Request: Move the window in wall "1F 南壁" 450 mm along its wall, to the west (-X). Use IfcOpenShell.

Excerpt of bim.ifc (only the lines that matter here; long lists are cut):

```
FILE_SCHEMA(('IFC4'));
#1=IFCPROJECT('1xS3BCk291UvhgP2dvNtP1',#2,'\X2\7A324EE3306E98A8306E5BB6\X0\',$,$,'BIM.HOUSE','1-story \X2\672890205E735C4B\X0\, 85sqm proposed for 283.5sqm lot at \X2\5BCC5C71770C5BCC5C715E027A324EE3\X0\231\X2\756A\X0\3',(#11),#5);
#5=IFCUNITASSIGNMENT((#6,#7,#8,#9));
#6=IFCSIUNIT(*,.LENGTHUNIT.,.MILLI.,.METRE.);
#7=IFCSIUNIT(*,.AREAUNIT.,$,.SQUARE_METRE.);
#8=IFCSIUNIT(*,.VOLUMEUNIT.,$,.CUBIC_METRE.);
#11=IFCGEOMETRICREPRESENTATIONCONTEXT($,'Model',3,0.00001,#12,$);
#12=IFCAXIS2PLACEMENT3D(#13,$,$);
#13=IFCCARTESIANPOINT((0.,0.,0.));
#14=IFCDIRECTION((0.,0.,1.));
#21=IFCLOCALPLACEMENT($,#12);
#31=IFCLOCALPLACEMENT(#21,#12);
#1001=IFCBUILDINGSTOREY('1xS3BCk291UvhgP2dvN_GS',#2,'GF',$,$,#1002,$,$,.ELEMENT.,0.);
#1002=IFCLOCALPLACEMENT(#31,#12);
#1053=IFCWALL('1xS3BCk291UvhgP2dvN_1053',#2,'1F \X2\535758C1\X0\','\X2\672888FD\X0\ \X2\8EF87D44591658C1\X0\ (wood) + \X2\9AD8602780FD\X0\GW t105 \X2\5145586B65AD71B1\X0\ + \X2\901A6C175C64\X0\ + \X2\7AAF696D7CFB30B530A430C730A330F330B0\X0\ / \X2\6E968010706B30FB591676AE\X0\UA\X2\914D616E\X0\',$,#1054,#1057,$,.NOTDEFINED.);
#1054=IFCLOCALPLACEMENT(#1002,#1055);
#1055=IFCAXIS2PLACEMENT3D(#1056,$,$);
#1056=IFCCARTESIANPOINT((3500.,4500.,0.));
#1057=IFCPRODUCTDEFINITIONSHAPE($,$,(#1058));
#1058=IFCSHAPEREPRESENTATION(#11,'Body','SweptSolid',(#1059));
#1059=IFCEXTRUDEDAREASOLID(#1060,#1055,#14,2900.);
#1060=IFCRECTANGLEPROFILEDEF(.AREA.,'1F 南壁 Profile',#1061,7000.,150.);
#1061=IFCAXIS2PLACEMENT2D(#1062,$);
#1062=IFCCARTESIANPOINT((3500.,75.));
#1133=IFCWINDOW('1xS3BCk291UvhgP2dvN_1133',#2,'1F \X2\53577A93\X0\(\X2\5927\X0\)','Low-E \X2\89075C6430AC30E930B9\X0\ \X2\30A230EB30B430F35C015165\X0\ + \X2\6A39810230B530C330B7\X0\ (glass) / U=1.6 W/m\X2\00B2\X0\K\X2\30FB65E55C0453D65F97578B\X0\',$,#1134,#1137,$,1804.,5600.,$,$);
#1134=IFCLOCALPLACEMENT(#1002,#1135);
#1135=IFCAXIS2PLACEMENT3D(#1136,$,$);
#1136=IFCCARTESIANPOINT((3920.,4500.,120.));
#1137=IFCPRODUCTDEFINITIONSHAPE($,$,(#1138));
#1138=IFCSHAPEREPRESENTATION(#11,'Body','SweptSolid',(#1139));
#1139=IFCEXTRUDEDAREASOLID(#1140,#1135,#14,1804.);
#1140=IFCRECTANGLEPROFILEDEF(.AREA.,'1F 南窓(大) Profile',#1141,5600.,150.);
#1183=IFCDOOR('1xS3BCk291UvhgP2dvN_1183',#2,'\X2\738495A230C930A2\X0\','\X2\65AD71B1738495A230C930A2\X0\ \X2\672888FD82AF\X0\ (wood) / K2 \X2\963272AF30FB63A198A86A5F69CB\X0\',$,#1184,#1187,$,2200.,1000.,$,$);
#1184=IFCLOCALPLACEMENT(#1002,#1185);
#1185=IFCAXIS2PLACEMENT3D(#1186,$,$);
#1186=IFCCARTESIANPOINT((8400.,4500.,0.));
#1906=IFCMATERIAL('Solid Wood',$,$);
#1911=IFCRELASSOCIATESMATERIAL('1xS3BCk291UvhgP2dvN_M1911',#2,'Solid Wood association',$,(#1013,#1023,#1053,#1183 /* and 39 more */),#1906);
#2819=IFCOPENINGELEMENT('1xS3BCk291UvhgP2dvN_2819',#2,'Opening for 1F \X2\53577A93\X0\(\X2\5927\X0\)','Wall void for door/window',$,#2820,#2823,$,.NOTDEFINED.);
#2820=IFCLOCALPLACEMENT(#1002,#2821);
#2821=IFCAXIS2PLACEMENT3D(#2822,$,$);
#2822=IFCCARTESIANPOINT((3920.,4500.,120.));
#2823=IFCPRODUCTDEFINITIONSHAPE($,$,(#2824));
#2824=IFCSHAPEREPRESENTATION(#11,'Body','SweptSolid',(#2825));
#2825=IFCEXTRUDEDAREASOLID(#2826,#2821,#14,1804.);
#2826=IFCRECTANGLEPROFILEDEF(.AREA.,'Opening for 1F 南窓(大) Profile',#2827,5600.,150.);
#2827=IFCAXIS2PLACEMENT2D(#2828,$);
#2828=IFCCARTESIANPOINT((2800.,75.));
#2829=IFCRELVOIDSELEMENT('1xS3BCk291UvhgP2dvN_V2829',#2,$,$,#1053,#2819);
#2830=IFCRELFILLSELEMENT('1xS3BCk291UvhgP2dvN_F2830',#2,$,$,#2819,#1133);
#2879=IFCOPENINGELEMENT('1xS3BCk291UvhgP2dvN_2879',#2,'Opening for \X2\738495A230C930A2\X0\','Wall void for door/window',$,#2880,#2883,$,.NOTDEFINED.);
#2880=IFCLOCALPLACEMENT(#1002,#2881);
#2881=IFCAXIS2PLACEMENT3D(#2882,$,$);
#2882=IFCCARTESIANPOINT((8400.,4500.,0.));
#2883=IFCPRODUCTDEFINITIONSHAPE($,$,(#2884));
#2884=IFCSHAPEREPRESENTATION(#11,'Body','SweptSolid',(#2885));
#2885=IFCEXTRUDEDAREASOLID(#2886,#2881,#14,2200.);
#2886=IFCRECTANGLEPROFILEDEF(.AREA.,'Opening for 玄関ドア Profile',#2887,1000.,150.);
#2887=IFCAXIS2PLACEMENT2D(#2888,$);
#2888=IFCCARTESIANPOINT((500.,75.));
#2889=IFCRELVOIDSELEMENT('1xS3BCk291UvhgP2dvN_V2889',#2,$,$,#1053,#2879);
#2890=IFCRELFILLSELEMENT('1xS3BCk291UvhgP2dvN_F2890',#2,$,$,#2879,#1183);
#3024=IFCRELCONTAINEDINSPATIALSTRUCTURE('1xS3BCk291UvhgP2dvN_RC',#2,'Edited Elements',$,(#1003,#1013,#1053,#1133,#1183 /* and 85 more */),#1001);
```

```python
import ifcopenshell
import ifcopenshell.api.geometry
import ifcopenshell.util.placement

model = ifcopenshell.open("bim.ifc")

window = model.by_guid("1xS3BCk291UvhgP2dvN_1133")
opening = window.FillsVoids[0].RelatingOpeningElement
wall = opening.VoidsElements[0].RelatingBuildingElement

wall_matrix = ifcopenshell.util.placement.get_local_placement(wall.ObjectPlacement)
shift = wall_matrix[:3, 0] * -450.0
before = ifcopenshell.util.placement.get_local_placement(window.ObjectPlacement)[:3, 3].copy()

# The window is not placed relative to its opening, so move both.
for product in (opening, window):
    matrix = ifcopenshell.util.placement.get_local_placement(product.ObjectPlacement)
    matrix[:3, 3] += shift
    ifcopenshell.api.geometry.edit_object_placement(model, product=product, matrix=matrix, is_si=False)

after = ifcopenshell.util.placement.get_local_placement(window.ObjectPlacement)[:3, 3]
print("window moved by", (after - before).round(3) + 0.0)

model.write("bim_updated.ifc")
```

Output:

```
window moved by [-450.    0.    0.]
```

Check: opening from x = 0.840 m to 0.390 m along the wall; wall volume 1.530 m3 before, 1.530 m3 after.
